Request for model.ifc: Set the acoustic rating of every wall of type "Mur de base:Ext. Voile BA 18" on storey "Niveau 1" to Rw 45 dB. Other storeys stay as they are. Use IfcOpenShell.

First a look at what the model holds.

```python
import ifcopenshell
import ifcopenshell.util.element

model = ifcopenshell.open("model.ifc")
print(model.schema)
storey = next(s for s in model.by_type("IfcBuildingStorey") if s.Name == "Niveau 1")
walls = [e for e in ifcopenshell.util.element.get_decomposition(storey) if e.is_a("IfcWall")]
seen = {}
for e in walls:
    element_type = ifcopenshell.util.element.get_type(e)
    key = (element_type.Name if element_type != e and element_type else None, ifcopenshell.util.element.get_pset(e, "Pset_WallCommon", "AcousticRating"))
    seen[key] = seen.get(key, 0) + 1
for (name, value), count in sorted(seen.items(), key=str):
    print(count, "x", name, "|", value)
```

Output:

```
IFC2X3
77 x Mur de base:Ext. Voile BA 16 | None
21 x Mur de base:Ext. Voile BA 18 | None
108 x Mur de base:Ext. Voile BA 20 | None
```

```python
import ifcopenshell
import ifcopenshell.api.pset
import ifcopenshell.util.element

model = ifcopenshell.open("model.ifc")

storey = next(s for s in model.by_type("IfcBuildingStorey") if s.Name == "Niveau 1")
walls = [e for e in ifcopenshell.util.element.get_decomposition(storey) if e.is_a("IfcWall")]

count = 0
for e in walls:
    element_type = ifcopenshell.util.element.get_type(e)
    if element_type in (None, e) or element_type.Name != "Mur de base:Ext. Voile BA 18":
        continue
    # add_pset returns the element's existing set when there is one.
    pset = ifcopenshell.api.pset.add_pset(model, product=e, name="Pset_WallCommon")
    ifcopenshell.api.pset.edit_pset(model, pset=pset, properties={"AcousticRating": "Rw 45 dB"})
    count += 1

print(count, "walls updated")

model.write("model_v2.ifc")
```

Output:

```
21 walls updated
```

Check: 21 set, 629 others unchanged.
